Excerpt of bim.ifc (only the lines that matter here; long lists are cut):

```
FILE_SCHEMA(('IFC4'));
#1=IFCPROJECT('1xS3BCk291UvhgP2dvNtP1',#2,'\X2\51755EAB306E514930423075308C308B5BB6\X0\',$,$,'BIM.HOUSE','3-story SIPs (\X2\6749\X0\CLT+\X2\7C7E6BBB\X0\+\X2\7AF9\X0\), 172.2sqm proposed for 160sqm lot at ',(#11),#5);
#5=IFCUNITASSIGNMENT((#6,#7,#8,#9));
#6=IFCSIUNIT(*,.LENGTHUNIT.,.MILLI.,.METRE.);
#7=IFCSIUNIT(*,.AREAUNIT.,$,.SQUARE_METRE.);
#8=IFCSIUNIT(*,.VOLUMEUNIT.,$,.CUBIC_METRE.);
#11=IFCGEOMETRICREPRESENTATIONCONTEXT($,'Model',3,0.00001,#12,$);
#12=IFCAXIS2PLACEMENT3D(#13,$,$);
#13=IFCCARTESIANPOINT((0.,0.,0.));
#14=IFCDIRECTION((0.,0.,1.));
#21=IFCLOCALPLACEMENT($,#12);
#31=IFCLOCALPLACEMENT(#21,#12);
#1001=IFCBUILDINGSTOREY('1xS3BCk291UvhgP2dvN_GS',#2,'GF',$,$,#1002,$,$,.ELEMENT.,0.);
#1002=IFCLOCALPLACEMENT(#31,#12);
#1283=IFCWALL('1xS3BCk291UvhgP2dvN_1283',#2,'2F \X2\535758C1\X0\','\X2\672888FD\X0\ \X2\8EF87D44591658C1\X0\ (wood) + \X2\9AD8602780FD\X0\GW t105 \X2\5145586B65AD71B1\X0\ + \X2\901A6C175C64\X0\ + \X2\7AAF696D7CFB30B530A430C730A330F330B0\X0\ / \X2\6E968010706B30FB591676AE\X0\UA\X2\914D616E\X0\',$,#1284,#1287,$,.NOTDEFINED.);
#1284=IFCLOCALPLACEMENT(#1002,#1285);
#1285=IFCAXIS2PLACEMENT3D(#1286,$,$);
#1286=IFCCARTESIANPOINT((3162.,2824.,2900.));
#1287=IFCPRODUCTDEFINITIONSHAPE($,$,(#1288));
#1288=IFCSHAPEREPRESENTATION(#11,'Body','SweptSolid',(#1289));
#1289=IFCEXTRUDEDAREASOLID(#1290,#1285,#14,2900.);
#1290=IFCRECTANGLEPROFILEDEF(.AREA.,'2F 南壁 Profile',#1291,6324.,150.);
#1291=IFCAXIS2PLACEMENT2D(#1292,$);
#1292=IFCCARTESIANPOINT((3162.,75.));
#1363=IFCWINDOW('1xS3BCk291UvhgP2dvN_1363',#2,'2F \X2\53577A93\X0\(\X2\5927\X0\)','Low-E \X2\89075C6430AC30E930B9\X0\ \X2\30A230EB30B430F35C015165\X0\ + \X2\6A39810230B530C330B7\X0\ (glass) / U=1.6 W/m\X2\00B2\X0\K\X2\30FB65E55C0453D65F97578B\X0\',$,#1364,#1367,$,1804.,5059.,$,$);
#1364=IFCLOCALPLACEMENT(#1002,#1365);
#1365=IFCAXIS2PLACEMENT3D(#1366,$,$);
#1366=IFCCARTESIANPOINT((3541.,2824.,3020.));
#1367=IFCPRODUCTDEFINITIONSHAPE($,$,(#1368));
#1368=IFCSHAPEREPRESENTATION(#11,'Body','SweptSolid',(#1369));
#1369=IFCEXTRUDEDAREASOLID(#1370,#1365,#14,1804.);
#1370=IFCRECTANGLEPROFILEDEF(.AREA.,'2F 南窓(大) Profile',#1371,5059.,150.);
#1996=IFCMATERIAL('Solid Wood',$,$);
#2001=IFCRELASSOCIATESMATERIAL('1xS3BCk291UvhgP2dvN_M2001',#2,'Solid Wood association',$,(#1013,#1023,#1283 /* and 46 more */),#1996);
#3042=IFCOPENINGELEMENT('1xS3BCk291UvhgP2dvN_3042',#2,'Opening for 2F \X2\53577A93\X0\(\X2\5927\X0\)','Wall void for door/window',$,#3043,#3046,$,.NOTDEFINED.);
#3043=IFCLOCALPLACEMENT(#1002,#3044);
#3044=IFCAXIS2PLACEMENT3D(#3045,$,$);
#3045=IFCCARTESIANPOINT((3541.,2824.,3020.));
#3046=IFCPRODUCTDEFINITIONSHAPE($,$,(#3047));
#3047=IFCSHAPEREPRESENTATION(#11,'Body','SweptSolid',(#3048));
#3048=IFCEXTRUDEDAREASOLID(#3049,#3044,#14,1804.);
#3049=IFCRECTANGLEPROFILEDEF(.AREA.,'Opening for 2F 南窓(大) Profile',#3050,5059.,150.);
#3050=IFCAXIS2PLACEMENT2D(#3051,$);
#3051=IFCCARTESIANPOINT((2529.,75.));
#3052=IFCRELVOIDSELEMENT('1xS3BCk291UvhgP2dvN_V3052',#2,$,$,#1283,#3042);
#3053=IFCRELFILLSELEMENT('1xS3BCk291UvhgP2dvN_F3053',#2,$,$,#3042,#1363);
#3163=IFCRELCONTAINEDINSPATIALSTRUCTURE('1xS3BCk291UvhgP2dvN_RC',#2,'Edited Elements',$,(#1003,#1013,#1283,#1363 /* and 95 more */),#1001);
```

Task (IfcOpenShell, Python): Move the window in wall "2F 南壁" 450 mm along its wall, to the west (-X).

```python
import ifcopenshell
import ifcopenshell.api.geometry
import ifcopenshell.util.placement

model = ifcopenshell.open("bim.ifc")

window = model.by_id(1363)
opening = window.FillsVoids[0].RelatingOpeningElement
wall = opening.VoidsElements[0].RelatingBuildingElement

wall_matrix = ifcopenshell.util.placement.get_local_placement(wall.ObjectPlacement)
shift = wall_matrix[:3, 0] * -450.0
before = ifcopenshell.util.placement.get_local_placement(window.ObjectPlacement)[:3, 3].copy()

# The window is not placed relative to its opening, so move both.
for product in (opening, window):
    matrix = ifcopenshell.util.placement.get_local_placement(product.ObjectPlacement)
    matrix[:3, 3] += shift
    ifcopenshell.api.geometry.edit_object_placement(model, product=product, matrix=matrix, is_si=False)

after = ifcopenshell.util.placement.get_local_placement(window.ObjectPlacement)[:3, 3]
print("window moved by", (after - before).round(3) + 0.0)

model.write("bim_updated.ifc")
```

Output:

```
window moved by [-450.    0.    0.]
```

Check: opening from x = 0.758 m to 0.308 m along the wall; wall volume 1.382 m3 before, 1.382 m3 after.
